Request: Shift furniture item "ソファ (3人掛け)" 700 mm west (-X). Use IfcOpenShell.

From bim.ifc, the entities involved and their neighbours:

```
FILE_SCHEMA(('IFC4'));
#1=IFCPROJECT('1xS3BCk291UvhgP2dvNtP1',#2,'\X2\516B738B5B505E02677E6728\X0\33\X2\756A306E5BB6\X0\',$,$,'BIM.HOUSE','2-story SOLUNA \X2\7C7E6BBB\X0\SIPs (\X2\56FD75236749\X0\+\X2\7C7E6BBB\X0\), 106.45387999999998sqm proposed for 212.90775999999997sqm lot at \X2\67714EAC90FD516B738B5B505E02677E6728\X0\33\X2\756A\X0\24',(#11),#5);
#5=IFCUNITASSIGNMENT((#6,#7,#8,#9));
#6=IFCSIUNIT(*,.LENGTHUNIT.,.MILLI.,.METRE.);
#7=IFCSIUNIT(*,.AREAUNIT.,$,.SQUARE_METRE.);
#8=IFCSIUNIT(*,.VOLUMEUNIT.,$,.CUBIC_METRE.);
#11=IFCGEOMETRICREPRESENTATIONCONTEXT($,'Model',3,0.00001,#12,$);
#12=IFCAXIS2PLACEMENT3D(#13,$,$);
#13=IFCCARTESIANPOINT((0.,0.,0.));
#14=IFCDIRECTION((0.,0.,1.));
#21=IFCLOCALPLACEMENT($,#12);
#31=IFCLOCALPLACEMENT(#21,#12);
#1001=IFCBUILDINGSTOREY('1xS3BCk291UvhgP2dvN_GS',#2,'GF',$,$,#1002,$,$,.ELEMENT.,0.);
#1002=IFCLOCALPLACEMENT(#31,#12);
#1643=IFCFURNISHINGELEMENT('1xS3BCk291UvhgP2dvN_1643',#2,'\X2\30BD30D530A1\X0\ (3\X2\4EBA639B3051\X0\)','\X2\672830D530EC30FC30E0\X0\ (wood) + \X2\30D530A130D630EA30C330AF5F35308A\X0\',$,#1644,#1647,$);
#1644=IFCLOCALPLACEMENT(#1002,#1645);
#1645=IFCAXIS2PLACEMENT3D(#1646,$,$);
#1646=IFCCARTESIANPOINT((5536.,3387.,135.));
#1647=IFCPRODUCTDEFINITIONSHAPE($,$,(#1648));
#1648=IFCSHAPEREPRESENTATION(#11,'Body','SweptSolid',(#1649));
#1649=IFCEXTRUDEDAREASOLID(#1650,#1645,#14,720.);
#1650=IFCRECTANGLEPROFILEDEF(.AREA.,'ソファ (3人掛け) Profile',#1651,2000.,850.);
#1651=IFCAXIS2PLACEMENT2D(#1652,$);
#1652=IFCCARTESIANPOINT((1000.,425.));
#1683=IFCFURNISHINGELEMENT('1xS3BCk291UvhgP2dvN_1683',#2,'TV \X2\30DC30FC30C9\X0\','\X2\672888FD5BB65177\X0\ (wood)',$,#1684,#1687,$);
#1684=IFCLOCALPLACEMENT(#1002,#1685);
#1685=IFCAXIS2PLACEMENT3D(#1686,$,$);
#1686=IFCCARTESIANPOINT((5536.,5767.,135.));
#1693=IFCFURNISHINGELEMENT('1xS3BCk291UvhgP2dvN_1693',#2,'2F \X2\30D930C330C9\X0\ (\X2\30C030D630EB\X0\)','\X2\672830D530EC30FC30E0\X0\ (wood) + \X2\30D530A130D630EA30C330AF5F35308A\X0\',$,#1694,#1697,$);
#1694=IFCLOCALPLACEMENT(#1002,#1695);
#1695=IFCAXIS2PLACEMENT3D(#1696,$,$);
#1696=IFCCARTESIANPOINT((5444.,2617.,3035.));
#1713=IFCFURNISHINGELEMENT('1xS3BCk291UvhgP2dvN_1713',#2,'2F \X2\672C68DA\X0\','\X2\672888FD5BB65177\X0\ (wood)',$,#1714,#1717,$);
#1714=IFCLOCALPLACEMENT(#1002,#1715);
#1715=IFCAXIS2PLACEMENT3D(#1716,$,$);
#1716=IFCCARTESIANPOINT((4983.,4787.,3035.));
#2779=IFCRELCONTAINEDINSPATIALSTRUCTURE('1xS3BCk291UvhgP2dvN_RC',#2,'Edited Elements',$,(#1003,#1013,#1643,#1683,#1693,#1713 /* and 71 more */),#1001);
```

```python
import ifcopenshell
import ifcopenshell.api.geometry
import ifcopenshell.util.placement
import ifcopenshell.util.unit

model = ifcopenshell.open("bim.ifc")
unit_scale = ifcopenshell.util.unit.calculate_unit_scale(model)

item = model.by_guid("1xS3BCk291UvhgP2dvN_1643")
matrix = ifcopenshell.util.placement.get_local_placement(item.ObjectPlacement)
matrix[0, 3] -= 0.7 / unit_scale
ifcopenshell.api.geometry.edit_object_placement(model, product=item, matrix=matrix, is_si=False)

print(ifcopenshell.util.placement.get_local_placement(item.ObjectPlacement).round(3) + 0.0)

model.write("bim_edited.ifc")
```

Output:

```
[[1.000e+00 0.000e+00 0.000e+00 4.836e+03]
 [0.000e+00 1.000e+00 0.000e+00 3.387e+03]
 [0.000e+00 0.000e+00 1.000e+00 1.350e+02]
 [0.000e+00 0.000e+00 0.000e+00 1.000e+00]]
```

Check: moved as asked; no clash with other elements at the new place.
